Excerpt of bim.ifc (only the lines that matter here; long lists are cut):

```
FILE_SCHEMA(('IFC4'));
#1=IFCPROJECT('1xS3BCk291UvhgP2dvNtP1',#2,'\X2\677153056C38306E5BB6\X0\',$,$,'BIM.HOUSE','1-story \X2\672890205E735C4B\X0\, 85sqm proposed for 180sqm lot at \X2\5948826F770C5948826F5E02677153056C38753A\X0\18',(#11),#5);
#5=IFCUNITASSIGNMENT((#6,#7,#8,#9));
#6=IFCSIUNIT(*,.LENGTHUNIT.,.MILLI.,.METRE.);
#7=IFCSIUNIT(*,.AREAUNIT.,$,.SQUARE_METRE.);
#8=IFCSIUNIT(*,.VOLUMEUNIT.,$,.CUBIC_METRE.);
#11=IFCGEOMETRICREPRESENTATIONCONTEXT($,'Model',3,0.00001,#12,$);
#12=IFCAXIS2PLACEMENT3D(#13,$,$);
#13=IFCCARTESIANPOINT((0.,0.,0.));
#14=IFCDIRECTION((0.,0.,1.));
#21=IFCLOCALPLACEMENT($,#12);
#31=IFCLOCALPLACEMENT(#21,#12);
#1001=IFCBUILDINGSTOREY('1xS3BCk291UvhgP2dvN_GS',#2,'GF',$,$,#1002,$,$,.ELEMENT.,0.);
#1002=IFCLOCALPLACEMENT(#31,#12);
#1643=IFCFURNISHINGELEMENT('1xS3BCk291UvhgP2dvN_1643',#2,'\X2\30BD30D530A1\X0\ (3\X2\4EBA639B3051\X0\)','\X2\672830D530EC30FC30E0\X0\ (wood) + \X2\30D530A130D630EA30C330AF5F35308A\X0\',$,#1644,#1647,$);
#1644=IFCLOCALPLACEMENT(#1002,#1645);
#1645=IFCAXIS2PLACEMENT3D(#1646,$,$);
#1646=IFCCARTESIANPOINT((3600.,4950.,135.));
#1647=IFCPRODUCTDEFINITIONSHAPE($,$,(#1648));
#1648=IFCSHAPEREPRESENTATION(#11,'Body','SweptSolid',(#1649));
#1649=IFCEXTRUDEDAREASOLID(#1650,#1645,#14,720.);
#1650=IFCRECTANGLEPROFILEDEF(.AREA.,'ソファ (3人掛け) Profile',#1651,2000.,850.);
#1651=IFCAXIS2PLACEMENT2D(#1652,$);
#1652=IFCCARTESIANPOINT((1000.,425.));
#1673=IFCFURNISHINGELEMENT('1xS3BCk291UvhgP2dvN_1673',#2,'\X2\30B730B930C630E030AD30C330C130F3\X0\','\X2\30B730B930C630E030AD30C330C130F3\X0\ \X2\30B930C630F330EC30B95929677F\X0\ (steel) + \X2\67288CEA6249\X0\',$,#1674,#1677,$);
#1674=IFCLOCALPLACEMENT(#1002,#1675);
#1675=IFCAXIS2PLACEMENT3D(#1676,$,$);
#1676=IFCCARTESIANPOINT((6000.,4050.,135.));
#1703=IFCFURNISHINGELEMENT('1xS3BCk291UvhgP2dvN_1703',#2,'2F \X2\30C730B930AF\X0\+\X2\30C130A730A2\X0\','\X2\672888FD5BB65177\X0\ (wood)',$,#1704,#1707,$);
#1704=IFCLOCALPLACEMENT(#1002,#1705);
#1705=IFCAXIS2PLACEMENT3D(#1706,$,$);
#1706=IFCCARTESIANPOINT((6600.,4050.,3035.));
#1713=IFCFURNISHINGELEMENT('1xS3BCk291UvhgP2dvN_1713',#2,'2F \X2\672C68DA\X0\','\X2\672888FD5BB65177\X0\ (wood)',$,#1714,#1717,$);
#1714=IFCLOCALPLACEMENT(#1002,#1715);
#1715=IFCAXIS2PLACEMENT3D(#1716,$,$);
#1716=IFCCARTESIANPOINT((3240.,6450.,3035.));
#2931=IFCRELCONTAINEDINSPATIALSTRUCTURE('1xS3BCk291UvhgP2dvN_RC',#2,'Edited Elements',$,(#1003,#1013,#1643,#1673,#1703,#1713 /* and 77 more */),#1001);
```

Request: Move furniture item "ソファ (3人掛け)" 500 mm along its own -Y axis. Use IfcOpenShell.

```python
import ifcopenshell
import ifcopenshell.api.geometry
import ifcopenshell.util.placement
import ifcopenshell.util.unit

model = ifcopenshell.open("bim.ifc")
unit_scale = ifcopenshell.util.unit.calculate_unit_scale(model)

item = model.by_guid("1xS3BCk291UvhgP2dvN_1643")
matrix = ifcopenshell.util.placement.get_local_placement(item.ObjectPlacement)
matrix[:3, 3] -= matrix[:3, 1] * 0.5 / unit_scale
ifcopenshell.api.geometry.edit_object_placement(model, product=item, matrix=matrix, is_si=False)

print(ifcopenshell.util.placement.get_local_placement(item.ObjectPlacement).round(3) + 0.0)

model.write("bim_updated.ifc")
```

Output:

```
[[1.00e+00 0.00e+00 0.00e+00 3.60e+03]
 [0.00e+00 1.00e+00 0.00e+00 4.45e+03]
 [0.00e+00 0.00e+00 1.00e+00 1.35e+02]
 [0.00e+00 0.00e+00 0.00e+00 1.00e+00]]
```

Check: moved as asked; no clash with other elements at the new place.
